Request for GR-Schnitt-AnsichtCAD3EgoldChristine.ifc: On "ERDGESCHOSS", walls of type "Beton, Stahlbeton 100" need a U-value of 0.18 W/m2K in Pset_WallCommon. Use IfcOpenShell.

First a look at what the model holds.

```python
import ifcopenshell
import ifcopenshell.util.element

model = ifcopenshell.open("GR-Schnitt-AnsichtCAD3EgoldChristine.ifc")
print(model.schema)
storey = next(s for s in model.by_type("IfcBuildingStorey") if s.Name == "ERDGESCHOSS")
walls = [e for e in ifcopenshell.util.element.get_decomposition(storey) if e.is_a("IfcWall")]
seen = {}
for e in walls:
    element_type = ifcopenshell.util.element.get_type(e)
    key = (element_type.Name if element_type != e and element_type else None, ifcopenshell.util.element.get_pset(e, "Pset_WallCommon", "ThermalTransmittance"))
    seen[key] = seen.get(key, 0) + 1
for (name, value), count in sorted(seen.items(), key=str):
    print(count, "x", name, "|", value)
```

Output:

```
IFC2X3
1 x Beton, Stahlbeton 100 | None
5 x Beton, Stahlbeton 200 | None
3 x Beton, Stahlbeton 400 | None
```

```python
import ifcopenshell
import ifcopenshell.api.pset
import ifcopenshell.util.element

model = ifcopenshell.open("GR-Schnitt-AnsichtCAD3EgoldChristine.ifc")

storey = next(s for s in model.by_type("IfcBuildingStorey") if s.Name == "ERDGESCHOSS")
walls = [e for e in ifcopenshell.util.element.get_decomposition(storey) if e.is_a("IfcWall")]

count = 0
for e in walls:
    element_type = ifcopenshell.util.element.get_type(e)
    if element_type in (None, e) or element_type.Name != "Beton, Stahlbeton 100":
        continue
    # add_pset returns the element's existing set when there is one.
    pset = ifcopenshell.api.pset.add_pset(model, product=e, name="Pset_WallCommon")
    ifcopenshell.api.pset.edit_pset(model, pset=pset, properties={"ThermalTransmittance": 0.18})
    count += 1

print(count, "walls updated")

model.write("GR-Schnitt-AnsichtCAD3EgoldChristine-out.ifc")
```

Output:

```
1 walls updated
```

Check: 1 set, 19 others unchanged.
